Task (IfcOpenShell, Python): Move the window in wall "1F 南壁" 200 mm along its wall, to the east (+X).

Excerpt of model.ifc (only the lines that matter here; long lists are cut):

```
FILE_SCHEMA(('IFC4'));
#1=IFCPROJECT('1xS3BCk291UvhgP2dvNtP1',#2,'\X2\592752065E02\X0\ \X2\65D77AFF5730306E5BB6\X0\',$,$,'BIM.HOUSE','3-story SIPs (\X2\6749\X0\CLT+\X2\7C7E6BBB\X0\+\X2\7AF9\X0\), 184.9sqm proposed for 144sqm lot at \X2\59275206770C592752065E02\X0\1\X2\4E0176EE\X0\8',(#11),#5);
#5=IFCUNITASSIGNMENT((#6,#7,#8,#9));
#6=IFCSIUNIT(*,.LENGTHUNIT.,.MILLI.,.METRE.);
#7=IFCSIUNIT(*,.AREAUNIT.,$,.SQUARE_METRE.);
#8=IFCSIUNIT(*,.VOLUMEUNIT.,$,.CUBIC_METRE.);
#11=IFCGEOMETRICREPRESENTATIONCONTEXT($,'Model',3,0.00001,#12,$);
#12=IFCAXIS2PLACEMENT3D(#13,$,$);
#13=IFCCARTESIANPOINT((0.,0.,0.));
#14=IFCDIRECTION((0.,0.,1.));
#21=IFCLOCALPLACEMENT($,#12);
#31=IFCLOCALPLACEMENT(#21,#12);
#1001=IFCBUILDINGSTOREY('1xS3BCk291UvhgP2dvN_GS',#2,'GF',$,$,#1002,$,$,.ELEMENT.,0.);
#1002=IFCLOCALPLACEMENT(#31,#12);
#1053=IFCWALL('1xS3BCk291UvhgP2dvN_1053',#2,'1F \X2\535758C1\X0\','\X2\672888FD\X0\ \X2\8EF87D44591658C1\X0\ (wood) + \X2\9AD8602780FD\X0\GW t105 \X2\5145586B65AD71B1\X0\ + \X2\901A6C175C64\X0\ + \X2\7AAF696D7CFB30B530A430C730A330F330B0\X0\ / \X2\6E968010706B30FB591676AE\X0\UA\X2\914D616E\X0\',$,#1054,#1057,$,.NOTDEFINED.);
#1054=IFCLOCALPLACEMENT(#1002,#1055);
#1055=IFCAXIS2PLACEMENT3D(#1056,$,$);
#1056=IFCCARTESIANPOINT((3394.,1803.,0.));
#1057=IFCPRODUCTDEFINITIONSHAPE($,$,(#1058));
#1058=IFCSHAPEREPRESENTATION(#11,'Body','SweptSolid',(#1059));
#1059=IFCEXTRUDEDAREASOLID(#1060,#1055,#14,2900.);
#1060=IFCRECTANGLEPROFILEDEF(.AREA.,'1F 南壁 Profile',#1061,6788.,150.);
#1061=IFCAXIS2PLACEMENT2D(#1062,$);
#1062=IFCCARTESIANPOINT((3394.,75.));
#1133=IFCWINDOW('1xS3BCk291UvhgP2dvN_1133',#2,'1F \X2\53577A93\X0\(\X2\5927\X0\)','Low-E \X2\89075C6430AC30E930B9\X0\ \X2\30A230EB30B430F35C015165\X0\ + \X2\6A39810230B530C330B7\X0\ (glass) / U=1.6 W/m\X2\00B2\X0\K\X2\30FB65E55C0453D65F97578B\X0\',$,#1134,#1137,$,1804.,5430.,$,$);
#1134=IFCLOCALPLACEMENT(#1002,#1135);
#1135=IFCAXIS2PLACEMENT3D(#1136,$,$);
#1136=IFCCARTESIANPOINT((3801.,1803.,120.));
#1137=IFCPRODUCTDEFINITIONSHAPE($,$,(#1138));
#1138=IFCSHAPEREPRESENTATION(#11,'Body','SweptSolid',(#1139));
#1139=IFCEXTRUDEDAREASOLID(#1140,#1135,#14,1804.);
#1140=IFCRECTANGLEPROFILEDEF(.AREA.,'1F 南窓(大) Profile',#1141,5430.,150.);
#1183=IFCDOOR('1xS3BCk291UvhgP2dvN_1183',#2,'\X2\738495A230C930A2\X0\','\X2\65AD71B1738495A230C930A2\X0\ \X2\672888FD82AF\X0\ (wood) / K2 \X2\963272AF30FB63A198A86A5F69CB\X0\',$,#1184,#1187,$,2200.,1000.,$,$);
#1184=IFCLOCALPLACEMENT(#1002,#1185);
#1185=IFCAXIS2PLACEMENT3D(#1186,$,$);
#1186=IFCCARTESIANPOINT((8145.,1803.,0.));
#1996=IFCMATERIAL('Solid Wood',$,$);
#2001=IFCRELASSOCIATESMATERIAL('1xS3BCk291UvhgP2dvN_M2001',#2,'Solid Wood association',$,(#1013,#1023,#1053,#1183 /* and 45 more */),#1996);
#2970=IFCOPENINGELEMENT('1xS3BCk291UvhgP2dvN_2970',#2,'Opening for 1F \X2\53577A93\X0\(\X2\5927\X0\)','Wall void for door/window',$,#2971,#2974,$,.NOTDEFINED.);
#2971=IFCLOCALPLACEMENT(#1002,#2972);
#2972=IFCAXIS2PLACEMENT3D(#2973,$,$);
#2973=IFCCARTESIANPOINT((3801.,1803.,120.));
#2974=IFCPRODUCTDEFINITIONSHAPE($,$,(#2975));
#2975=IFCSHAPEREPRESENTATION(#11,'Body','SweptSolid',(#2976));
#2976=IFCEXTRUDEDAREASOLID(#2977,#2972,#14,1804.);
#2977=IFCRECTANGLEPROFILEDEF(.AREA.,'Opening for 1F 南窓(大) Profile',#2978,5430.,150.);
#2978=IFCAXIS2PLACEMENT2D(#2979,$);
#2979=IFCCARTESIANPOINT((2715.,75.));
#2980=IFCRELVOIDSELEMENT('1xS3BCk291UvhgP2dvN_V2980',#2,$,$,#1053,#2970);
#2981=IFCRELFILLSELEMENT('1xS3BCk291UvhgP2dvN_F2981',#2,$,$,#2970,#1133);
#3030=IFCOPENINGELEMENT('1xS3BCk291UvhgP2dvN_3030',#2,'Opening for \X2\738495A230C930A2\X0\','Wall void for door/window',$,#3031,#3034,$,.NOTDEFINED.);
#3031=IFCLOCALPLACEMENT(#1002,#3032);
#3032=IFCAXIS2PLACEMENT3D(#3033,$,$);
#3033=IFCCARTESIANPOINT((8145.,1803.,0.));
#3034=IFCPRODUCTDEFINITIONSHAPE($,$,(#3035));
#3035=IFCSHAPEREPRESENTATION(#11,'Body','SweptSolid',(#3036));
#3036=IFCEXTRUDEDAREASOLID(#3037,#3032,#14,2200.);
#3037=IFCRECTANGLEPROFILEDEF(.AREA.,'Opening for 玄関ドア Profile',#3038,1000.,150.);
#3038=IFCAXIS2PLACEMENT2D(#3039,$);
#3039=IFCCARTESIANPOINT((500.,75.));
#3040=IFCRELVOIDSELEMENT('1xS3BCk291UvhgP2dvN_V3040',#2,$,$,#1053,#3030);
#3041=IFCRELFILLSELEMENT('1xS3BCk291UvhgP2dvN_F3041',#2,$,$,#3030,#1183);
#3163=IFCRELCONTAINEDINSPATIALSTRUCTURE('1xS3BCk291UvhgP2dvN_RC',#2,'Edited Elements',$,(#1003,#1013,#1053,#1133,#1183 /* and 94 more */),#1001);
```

```python
import ifcopenshell
import ifcopenshell.api.geometry
import ifcopenshell.util.placement

model = ifcopenshell.open("model.ifc")

window = model.by_guid("1xS3BCk291UvhgP2dvN_1133")
opening = window.FillsVoids[0].RelatingOpeningElement
wall = opening.VoidsElements[0].RelatingBuildingElement

wall_matrix = ifcopenshell.util.placement.get_local_placement(wall.ObjectPlacement)
shift = wall_matrix[:3, 0] * 200.0
before = ifcopenshell.util.placement.get_local_placement(window.ObjectPlacement)[:3, 3].copy()

# The window is not placed relative to its opening, so move both.
for product in (opening, window):
    matrix = ifcopenshell.util.placement.get_local_placement(product.ObjectPlacement)
    matrix[:3, 3] += shift
    ifcopenshell.api.geometry.edit_object_placement(model, product=product, matrix=matrix, is_si=False)

after = ifcopenshell.util.placement.get_local_placement(window.ObjectPlacement)[:3, 3]
print("window moved by", (after - before).round(3) + 0.0)

model.write("model-out.ifc")
```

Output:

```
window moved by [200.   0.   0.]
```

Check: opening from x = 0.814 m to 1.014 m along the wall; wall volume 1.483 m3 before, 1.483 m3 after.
